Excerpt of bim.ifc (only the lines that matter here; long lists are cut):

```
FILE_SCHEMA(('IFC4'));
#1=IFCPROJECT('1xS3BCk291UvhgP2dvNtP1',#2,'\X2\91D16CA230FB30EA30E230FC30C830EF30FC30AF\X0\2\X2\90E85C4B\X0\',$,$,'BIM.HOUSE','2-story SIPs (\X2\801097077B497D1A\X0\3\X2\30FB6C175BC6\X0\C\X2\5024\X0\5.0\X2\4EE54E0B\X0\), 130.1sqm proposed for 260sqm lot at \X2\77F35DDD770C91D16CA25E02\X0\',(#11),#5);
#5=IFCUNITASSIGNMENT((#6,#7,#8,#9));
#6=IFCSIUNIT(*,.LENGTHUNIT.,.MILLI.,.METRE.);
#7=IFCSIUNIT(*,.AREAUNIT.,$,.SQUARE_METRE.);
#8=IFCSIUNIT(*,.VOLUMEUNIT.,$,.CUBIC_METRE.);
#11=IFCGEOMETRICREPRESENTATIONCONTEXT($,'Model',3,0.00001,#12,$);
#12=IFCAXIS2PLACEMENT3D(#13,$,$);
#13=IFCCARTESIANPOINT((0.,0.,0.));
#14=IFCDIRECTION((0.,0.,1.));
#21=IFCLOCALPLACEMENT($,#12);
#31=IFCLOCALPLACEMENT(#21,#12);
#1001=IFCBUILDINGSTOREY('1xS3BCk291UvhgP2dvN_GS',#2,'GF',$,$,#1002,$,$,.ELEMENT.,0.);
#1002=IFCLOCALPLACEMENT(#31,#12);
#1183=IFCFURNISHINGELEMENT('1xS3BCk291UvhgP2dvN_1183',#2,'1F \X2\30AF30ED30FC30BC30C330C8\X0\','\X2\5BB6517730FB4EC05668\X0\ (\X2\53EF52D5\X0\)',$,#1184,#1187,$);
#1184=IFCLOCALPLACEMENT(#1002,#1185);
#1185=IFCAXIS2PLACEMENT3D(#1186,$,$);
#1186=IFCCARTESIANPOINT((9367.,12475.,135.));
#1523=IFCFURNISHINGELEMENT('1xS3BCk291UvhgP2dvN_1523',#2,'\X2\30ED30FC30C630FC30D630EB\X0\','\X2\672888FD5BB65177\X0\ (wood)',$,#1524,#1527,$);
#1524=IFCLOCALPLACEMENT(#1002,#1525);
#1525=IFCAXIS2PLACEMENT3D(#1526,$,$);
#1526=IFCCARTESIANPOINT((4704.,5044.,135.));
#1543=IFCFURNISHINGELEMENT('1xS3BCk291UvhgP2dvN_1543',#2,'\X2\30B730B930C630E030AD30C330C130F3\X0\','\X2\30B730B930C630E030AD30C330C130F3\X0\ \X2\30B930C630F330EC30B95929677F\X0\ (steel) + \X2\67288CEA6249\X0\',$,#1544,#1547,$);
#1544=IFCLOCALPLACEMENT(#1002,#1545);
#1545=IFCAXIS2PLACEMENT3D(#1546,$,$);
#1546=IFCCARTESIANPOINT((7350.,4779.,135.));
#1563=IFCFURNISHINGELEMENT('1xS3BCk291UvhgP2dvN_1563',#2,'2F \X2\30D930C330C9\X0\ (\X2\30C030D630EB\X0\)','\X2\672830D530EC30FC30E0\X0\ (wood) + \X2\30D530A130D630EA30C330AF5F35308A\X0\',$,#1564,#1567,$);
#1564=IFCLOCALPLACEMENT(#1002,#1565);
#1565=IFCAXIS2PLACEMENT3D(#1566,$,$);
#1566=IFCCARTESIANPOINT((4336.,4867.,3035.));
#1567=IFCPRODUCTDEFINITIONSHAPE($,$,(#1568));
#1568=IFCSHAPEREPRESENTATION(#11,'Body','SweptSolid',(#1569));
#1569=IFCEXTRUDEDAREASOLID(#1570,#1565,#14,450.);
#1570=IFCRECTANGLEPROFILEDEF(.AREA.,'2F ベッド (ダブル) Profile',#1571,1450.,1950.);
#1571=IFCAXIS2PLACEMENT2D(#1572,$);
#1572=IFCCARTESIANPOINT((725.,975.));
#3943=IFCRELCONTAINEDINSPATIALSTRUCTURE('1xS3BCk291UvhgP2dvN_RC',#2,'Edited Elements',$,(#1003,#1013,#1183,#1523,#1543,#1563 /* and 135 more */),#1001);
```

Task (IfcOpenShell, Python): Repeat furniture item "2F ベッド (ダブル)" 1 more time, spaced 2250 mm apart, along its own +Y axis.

```python
import ifcopenshell
import ifcopenshell.api.geometry
import ifcopenshell.api.root
import ifcopenshell.util.element
import ifcopenshell.util.placement
import ifcopenshell.util.unit

model = ifcopenshell.open("bim.ifc")
unit_scale = ifcopenshell.util.unit.calculate_unit_scale(model)


def reuse_history(source, copy):
    """copy_class also copies each property set's owner history, people and application; keep the originals."""
    for rel in copy.IsDefinedBy:
        if rel.is_a("IfcRelDefinesByProperties") and (history := rel.RelatingPropertyDefinition.OwnerHistory):
            rel.RelatingPropertyDefinition.OwnerHistory = source.OwnerHistory
            ifcopenshell.util.element.remove_deep2(model, history)


source = model.by_guid("1xS3BCk291UvhgP2dvN_1563")
base = ifcopenshell.util.placement.get_local_placement(source.ObjectPlacement)
step = base[:3, 1] * 2.25 / unit_scale

for i in range(1, 2):
    copy = ifcopenshell.api.root.copy_class(model, product=source)
    copy.Representation = ifcopenshell.util.element.copy_deep(
        model, source.Representation, exclude=["IfcGeometricRepresentationContext", "IfcRepresentationMap"]
    )
    reuse_history(source, copy)
    matrix = base.copy()
    matrix[:3, 3] += i * step
    print("added at", matrix[:3, 3].round(3) + 0.0)
    ifcopenshell.api.geometry.edit_object_placement(model, product=copy, matrix=matrix, is_si=False)

model.write("bim_updated.ifc")
```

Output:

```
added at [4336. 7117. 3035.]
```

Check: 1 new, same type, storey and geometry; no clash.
